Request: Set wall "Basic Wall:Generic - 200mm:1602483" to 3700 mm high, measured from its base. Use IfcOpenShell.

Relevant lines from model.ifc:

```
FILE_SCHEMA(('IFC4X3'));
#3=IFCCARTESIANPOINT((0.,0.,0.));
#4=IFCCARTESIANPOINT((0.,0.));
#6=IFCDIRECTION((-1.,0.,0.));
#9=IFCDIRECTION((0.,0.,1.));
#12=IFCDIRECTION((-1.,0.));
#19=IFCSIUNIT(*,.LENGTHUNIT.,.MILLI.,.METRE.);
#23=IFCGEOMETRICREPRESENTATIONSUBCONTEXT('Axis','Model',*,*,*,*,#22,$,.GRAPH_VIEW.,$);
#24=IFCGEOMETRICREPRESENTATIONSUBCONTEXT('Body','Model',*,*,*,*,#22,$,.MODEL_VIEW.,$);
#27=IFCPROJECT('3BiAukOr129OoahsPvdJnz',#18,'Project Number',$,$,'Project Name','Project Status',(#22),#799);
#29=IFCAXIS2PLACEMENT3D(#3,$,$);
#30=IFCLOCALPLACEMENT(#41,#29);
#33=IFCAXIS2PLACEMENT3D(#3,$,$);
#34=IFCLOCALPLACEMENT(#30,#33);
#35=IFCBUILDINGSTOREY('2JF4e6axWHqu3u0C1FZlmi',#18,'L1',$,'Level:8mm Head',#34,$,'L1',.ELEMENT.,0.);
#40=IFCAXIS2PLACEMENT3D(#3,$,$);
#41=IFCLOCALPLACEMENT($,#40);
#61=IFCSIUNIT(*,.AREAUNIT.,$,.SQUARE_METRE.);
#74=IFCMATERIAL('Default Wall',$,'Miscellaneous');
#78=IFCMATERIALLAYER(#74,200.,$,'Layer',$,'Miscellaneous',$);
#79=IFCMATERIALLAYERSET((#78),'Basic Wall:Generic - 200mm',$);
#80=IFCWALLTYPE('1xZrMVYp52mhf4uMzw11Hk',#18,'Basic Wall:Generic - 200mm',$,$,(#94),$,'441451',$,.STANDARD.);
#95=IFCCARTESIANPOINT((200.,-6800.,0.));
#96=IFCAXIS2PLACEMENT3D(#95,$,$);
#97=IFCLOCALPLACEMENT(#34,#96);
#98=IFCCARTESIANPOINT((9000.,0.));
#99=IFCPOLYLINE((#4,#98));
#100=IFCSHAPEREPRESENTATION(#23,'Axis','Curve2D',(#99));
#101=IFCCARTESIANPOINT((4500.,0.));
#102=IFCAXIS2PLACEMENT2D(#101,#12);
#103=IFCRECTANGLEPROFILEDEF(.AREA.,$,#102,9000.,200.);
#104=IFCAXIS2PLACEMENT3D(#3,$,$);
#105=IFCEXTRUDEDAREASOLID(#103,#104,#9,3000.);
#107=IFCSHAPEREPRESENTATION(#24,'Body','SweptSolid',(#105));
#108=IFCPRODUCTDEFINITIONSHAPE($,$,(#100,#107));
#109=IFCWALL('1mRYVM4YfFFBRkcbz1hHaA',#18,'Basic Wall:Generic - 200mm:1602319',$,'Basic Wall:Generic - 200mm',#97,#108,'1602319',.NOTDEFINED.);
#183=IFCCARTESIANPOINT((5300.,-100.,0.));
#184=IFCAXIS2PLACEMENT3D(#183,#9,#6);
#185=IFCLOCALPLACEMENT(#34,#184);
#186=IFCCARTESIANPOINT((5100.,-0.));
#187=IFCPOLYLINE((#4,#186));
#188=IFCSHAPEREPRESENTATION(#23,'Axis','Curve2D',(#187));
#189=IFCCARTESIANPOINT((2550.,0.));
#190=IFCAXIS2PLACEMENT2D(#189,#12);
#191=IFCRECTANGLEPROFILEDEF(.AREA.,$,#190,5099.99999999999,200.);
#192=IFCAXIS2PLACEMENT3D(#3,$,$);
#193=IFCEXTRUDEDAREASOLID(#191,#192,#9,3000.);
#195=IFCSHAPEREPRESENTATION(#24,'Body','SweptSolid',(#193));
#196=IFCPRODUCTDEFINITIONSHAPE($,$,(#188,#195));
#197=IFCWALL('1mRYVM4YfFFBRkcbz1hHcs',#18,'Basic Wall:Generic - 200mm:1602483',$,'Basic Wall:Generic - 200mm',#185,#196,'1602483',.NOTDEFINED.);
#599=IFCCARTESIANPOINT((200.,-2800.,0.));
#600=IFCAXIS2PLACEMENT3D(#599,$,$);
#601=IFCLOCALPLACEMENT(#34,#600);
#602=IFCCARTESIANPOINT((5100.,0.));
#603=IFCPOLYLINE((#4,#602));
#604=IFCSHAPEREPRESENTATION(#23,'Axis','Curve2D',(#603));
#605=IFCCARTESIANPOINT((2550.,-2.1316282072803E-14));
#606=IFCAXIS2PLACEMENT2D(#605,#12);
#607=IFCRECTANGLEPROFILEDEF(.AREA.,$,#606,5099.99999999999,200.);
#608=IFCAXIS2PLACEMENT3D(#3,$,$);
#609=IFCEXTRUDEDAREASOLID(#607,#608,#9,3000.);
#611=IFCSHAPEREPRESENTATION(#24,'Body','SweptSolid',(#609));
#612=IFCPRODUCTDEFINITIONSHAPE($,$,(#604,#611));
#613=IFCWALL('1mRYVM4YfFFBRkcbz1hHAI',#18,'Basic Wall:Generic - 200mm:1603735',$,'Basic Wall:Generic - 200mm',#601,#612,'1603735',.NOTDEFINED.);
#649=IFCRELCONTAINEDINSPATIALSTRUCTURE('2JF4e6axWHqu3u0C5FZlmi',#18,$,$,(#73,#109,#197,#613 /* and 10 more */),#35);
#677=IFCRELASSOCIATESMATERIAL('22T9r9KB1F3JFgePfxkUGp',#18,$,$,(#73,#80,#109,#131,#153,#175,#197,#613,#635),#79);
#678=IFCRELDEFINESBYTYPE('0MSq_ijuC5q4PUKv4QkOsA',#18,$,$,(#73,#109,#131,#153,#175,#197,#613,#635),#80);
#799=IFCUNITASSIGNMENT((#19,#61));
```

```python
import ifcopenshell
import ifcopenshell.geom
import ifcopenshell.util.representation
import ifcopenshell.util.shape
import ifcopenshell.util.unit

model = ifcopenshell.open("model.ifc")
unit_scale = ifcopenshell.util.unit.calculate_unit_scale(model)
settings = ifcopenshell.geom.settings()


def volume(element):
    """Net volume in cubic metres, openings subtracted."""
    shape = ifcopenshell.geom.create_shape(settings, element)
    return ifcopenshell.util.shape.get_volume(shape.geometry)


wall = model.by_guid("1mRYVM4YfFFBRkcbz1hHcs")
before = volume(wall)

body = ifcopenshell.util.representation.get_representation(wall, "Model", "Body")
solid = body.Items[0]
old_height = solid.Depth
solid.Depth = 3.7 / unit_scale
after = volume(wall)

print(f"height {old_height:g} -> {solid.Depth:g}, volume {before:.3f} -> {after:.3f} m3")

model.write("model-out.ifc")
```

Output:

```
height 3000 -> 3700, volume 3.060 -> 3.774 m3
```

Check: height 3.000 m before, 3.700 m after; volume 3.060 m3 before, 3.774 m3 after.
